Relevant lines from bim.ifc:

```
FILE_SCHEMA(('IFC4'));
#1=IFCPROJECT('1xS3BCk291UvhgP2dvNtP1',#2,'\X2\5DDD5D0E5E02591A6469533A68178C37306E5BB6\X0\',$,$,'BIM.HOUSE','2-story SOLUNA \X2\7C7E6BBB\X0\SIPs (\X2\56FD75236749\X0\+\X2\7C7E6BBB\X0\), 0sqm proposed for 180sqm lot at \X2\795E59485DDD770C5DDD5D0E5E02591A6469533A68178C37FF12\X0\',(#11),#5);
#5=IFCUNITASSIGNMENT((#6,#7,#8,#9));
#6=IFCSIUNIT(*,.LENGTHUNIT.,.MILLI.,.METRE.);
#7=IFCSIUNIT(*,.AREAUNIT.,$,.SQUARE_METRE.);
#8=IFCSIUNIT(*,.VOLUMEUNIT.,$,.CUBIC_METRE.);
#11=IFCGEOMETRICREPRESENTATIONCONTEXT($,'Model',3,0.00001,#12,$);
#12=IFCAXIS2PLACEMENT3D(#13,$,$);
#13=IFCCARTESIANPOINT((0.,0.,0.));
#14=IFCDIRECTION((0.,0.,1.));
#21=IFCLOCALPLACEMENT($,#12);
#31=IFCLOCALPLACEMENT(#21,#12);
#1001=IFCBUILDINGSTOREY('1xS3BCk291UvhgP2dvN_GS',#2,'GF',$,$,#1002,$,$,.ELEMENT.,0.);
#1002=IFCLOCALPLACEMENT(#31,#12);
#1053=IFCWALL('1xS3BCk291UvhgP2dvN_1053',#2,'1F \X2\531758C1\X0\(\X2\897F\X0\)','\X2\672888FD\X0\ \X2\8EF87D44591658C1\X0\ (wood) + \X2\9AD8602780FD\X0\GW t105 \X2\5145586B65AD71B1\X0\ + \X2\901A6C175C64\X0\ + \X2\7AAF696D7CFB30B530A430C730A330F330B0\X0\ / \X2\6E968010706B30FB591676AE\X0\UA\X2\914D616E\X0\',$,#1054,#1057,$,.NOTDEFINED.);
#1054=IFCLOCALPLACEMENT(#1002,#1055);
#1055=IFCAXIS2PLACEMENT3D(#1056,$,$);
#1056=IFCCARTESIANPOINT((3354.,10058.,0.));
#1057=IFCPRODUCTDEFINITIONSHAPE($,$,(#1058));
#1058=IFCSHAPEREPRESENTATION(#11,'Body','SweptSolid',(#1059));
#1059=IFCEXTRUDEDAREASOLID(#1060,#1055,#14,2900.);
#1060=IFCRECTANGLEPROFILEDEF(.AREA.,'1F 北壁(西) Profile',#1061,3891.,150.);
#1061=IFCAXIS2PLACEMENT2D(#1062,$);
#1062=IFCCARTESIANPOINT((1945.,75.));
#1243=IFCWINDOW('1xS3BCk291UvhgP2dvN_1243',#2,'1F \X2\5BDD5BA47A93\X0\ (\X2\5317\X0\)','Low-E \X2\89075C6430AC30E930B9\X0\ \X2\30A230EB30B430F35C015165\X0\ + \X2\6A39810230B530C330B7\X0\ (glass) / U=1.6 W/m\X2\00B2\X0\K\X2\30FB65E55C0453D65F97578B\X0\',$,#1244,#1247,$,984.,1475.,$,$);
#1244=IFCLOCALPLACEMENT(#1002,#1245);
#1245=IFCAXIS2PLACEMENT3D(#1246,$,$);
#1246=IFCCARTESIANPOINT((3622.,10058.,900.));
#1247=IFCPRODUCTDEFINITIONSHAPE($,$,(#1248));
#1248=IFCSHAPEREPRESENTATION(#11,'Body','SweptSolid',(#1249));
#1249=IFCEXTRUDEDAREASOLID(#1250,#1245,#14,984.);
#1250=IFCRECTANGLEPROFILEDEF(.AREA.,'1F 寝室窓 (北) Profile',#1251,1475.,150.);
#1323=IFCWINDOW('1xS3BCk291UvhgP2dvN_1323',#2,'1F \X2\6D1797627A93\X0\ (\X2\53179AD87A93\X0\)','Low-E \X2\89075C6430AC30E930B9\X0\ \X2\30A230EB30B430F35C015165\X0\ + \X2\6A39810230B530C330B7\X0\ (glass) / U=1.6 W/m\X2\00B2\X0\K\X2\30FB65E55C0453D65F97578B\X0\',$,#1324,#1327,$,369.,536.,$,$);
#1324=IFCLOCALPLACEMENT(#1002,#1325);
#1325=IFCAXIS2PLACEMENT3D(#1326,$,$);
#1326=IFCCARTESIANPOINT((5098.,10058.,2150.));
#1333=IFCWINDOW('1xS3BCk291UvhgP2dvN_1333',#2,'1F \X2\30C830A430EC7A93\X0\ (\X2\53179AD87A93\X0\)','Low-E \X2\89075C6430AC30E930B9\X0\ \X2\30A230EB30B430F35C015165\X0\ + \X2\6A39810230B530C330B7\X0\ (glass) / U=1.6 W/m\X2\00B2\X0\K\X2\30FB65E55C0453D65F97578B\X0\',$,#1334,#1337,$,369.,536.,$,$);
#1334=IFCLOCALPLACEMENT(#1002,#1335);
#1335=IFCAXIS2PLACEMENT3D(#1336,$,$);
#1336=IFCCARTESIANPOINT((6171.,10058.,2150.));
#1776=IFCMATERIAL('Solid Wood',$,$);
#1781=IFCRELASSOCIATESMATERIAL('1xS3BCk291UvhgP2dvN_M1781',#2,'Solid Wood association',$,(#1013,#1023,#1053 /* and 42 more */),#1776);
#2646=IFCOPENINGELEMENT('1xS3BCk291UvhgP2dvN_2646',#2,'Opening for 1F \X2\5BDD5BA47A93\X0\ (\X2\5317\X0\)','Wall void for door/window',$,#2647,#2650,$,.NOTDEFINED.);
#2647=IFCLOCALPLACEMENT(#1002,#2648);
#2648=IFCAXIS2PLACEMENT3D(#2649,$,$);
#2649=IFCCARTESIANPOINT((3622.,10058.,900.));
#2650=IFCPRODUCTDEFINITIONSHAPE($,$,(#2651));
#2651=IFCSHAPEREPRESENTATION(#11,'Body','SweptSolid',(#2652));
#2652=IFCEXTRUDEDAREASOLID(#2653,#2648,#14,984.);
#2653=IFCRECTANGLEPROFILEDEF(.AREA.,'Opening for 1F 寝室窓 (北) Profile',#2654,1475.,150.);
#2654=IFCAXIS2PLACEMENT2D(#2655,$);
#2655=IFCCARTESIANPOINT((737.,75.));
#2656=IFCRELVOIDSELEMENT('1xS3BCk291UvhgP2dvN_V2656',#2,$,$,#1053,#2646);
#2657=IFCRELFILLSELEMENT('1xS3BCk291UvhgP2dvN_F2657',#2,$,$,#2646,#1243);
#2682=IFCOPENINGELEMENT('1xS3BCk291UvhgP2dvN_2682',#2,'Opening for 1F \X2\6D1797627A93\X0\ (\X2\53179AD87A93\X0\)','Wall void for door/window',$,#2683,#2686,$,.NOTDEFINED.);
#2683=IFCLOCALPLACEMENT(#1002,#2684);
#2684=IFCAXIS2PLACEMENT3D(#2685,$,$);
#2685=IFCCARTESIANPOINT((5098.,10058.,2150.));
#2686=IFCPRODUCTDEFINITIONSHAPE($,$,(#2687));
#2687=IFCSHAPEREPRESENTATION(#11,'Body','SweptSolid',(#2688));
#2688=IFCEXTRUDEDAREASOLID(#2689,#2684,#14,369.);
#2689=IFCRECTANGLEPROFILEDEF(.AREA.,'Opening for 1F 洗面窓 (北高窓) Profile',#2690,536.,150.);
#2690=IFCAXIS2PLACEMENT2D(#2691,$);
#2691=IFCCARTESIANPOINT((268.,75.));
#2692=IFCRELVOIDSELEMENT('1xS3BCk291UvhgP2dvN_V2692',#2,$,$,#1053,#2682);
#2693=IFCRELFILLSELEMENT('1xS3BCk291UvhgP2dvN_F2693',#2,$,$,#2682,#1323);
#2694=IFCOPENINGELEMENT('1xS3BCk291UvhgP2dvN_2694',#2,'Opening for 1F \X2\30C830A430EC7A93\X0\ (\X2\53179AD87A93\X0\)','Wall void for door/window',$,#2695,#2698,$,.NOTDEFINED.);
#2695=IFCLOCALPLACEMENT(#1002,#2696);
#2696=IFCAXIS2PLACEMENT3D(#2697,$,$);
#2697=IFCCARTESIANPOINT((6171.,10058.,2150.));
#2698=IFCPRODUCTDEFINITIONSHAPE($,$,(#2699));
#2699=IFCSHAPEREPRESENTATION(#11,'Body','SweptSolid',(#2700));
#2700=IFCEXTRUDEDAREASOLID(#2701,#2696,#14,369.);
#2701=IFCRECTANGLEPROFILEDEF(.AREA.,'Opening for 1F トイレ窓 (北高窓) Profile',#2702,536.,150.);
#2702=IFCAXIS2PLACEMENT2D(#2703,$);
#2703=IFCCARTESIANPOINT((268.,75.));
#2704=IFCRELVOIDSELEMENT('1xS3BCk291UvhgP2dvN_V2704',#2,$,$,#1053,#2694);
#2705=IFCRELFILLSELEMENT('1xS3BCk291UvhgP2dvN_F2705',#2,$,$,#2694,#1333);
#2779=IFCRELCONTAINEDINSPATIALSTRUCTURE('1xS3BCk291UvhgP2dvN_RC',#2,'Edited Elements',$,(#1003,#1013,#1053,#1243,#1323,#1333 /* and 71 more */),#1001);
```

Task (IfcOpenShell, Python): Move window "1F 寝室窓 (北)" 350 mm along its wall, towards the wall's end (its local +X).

```python
import ifcopenshell
import ifcopenshell.api.geometry
import ifcopenshell.util.placement

model = ifcopenshell.open("bim.ifc")

window = model.by_id(1243)
opening = window.FillsVoids[0].RelatingOpeningElement
wall = opening.VoidsElements[0].RelatingBuildingElement

wall_matrix = ifcopenshell.util.placement.get_local_placement(wall.ObjectPlacement)
shift = wall_matrix[:3, 0] * 350.0
before = ifcopenshell.util.placement.get_local_placement(window.ObjectPlacement)[:3, 3].copy()

# The window is not placed relative to its opening, so move both.
for product in (opening, window):
    matrix = ifcopenshell.util.placement.get_local_placement(product.ObjectPlacement)
    matrix[:3, 3] += shift
    ifcopenshell.api.geometry.edit_object_placement(model, product=product, matrix=matrix, is_si=False)

after = ifcopenshell.util.placement.get_local_placement(window.ObjectPlacement)[:3, 3]
print("window moved by", (after - before).round(3) + 0.0)

model.write("bim_rev.ifc")
```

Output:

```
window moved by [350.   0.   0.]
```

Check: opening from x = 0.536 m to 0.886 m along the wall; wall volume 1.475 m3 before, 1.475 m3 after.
